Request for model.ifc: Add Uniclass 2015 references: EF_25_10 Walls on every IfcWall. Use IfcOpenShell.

First a look at what the model holds.

```python
import ifcopenshell

model = ifcopenshell.open("model.ifc")
print(model.schema)
print("classifications:", [c.Name for c in model.by_type("IfcClassification")])
for ifc_class in ("IfcDoor", "IfcRoof", "IfcStair", "IfcWall", "IfcWindow"):
    print(ifc_class, len(model.by_type(ifc_class)))
```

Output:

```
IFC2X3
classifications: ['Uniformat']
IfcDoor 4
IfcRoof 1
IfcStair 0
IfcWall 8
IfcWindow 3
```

```python
import ifcopenshell
import ifcopenshell.api.classification

model = ifcopenshell.open("model.ifc")

# IFC2X3 requires Source and Edition and has no link from the project to the system.
system = model.create_entity("IfcClassification", Source="NBS", Edition="2015", Name="Uniclass 2015")

codes = {
    "IfcWall": ("EF_25_10", "Walls"),
}
for ifc_class, (code, name) in codes.items():
    products = model.by_type(ifc_class)
    ifcopenshell.api.classification.add_reference(
        model, products=products, classification=system, identification=code, name=name
    )
    print(code, len(products))

model.write("model_edited.ifc")
```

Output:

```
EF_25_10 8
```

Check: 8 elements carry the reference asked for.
